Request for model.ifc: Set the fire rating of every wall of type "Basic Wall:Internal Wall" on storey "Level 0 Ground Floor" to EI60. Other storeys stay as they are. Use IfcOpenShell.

First a look at what the model holds.

```python
import ifcopenshell
import ifcopenshell.util.element

model = ifcopenshell.open("model.ifc")
print(model.schema)
storey = next(s for s in model.by_type("IfcBuildingStorey") if s.Name == "Level 0 Ground Floor")
walls = [e for e in ifcopenshell.util.element.get_decomposition(storey) if e.is_a("IfcWall")]
seen = {}
for e in walls:
    element_type = ifcopenshell.util.element.get_type(e)
    key = (element_type.Name if element_type != e and element_type else None, ifcopenshell.util.element.get_pset(e, "Pset_WallCommon", "FireRating"))
    seen[key] = seen.get(key, 0) + 1
for (name, value), count in sorted(seen.items(), key=str):
    print(count, "x", name, "|", value)
```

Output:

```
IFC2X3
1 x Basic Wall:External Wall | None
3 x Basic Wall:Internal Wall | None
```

```python
import ifcopenshell
import ifcopenshell.api.pset
import ifcopenshell.util.element

model = ifcopenshell.open("model.ifc")

storey = next(s for s in model.by_type("IfcBuildingStorey") if s.Name == "Level 0 Ground Floor")
walls = [e for e in ifcopenshell.util.element.get_decomposition(storey) if e.is_a("IfcWall")]

count = 0
for e in walls:
    element_type = ifcopenshell.util.element.get_type(e)
    if element_type in (None, e) or element_type.Name != "Basic Wall:Internal Wall":
        continue
    # add_pset returns the element's existing set when there is one.
    pset = ifcopenshell.api.pset.add_pset(model, product=e, name="Pset_WallCommon")
    ifcopenshell.api.pset.edit_pset(model, pset=pset, properties={"FireRating": "EI60"})
    count += 1

print(count, "walls updated")

model.write("model-out.ifc")
```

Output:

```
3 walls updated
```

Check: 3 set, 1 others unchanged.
